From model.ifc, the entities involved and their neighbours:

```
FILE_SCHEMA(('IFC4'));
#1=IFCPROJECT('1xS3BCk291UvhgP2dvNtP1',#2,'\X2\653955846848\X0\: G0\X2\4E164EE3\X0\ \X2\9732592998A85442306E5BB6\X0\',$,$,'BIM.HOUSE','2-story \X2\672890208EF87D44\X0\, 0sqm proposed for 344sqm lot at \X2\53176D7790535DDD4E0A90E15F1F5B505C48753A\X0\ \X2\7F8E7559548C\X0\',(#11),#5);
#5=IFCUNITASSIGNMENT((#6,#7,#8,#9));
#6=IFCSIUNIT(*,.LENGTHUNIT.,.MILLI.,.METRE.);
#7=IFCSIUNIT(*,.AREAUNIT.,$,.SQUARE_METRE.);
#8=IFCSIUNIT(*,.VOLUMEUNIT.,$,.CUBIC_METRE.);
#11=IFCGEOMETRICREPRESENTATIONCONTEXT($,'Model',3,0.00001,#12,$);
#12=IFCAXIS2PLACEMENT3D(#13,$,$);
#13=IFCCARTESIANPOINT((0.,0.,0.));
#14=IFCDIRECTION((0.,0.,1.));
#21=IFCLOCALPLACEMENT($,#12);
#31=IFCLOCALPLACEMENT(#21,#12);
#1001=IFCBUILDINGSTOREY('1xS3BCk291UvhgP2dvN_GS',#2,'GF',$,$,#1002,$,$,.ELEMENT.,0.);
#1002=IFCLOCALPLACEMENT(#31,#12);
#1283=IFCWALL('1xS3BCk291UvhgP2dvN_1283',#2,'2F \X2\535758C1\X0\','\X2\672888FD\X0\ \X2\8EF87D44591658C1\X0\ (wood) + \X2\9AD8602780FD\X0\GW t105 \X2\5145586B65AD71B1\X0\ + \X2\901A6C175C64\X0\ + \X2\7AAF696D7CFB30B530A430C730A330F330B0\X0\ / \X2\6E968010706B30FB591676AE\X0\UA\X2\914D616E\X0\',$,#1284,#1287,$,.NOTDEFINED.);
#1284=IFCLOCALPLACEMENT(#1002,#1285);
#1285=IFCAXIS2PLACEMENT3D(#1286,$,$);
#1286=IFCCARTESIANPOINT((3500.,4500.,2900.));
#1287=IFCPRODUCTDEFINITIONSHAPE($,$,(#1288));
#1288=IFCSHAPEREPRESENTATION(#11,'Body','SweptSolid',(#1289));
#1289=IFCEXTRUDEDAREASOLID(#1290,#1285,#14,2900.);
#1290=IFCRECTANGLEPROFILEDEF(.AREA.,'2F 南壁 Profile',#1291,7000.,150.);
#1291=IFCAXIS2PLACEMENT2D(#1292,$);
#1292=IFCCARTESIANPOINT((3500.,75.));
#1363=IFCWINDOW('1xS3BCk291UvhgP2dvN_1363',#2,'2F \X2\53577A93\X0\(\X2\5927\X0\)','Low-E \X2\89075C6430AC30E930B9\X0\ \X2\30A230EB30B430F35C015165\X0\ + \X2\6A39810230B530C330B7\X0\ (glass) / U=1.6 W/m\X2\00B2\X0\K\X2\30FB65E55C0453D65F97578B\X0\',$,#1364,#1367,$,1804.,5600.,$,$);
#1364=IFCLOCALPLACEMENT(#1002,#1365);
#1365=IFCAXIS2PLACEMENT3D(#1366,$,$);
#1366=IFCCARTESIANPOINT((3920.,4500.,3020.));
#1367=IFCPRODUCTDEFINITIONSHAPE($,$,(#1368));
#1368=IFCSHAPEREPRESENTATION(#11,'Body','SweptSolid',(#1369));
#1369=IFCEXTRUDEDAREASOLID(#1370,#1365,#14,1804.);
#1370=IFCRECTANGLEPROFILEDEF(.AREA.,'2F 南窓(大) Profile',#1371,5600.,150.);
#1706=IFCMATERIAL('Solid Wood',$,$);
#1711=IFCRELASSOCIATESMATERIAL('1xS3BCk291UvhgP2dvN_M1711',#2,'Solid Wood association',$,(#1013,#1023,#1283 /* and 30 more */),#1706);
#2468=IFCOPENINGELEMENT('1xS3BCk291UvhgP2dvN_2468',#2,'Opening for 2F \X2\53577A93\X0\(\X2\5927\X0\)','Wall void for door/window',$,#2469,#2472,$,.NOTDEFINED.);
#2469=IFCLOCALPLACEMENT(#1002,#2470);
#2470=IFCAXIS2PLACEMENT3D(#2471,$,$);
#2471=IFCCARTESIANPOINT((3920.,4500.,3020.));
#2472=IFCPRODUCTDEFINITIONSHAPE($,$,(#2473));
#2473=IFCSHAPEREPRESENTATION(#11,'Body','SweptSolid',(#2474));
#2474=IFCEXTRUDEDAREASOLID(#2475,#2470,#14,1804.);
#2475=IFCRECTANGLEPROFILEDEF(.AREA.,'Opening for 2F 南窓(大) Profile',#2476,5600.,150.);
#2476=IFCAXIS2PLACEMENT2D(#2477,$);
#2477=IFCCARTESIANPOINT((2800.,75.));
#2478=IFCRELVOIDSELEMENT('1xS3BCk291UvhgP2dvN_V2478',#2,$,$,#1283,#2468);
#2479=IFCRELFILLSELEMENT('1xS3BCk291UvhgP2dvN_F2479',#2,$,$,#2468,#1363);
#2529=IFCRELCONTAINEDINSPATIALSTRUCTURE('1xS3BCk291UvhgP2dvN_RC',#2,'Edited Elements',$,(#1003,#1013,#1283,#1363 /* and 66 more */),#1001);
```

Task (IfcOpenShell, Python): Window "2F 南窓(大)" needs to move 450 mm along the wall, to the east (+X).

```python
import ifcopenshell
import ifcopenshell.api.geometry
import ifcopenshell.util.placement

model = ifcopenshell.open("model.ifc")

window = model.by_id(1363)
opening = window.FillsVoids[0].RelatingOpeningElement
wall = opening.VoidsElements[0].RelatingBuildingElement

wall_matrix = ifcopenshell.util.placement.get_local_placement(wall.ObjectPlacement)
shift = wall_matrix[:3, 0] * 450.0
before = ifcopenshell.util.placement.get_local_placement(window.ObjectPlacement)[:3, 3].copy()

# The window is not placed relative to its opening, so move both.
for product in (opening, window):
    matrix = ifcopenshell.util.placement.get_local_placement(product.ObjectPlacement)
    matrix[:3, 3] += shift
    ifcopenshell.api.geometry.edit_object_placement(model, product=product, matrix=matrix, is_si=False)

after = ifcopenshell.util.placement.get_local_placement(window.ObjectPlacement)[:3, 3]
print("window moved by", (after - before).round(3) + 0.0)

model.write("model_updated.ifc")
```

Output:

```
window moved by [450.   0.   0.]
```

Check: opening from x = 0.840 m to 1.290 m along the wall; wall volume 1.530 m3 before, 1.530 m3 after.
